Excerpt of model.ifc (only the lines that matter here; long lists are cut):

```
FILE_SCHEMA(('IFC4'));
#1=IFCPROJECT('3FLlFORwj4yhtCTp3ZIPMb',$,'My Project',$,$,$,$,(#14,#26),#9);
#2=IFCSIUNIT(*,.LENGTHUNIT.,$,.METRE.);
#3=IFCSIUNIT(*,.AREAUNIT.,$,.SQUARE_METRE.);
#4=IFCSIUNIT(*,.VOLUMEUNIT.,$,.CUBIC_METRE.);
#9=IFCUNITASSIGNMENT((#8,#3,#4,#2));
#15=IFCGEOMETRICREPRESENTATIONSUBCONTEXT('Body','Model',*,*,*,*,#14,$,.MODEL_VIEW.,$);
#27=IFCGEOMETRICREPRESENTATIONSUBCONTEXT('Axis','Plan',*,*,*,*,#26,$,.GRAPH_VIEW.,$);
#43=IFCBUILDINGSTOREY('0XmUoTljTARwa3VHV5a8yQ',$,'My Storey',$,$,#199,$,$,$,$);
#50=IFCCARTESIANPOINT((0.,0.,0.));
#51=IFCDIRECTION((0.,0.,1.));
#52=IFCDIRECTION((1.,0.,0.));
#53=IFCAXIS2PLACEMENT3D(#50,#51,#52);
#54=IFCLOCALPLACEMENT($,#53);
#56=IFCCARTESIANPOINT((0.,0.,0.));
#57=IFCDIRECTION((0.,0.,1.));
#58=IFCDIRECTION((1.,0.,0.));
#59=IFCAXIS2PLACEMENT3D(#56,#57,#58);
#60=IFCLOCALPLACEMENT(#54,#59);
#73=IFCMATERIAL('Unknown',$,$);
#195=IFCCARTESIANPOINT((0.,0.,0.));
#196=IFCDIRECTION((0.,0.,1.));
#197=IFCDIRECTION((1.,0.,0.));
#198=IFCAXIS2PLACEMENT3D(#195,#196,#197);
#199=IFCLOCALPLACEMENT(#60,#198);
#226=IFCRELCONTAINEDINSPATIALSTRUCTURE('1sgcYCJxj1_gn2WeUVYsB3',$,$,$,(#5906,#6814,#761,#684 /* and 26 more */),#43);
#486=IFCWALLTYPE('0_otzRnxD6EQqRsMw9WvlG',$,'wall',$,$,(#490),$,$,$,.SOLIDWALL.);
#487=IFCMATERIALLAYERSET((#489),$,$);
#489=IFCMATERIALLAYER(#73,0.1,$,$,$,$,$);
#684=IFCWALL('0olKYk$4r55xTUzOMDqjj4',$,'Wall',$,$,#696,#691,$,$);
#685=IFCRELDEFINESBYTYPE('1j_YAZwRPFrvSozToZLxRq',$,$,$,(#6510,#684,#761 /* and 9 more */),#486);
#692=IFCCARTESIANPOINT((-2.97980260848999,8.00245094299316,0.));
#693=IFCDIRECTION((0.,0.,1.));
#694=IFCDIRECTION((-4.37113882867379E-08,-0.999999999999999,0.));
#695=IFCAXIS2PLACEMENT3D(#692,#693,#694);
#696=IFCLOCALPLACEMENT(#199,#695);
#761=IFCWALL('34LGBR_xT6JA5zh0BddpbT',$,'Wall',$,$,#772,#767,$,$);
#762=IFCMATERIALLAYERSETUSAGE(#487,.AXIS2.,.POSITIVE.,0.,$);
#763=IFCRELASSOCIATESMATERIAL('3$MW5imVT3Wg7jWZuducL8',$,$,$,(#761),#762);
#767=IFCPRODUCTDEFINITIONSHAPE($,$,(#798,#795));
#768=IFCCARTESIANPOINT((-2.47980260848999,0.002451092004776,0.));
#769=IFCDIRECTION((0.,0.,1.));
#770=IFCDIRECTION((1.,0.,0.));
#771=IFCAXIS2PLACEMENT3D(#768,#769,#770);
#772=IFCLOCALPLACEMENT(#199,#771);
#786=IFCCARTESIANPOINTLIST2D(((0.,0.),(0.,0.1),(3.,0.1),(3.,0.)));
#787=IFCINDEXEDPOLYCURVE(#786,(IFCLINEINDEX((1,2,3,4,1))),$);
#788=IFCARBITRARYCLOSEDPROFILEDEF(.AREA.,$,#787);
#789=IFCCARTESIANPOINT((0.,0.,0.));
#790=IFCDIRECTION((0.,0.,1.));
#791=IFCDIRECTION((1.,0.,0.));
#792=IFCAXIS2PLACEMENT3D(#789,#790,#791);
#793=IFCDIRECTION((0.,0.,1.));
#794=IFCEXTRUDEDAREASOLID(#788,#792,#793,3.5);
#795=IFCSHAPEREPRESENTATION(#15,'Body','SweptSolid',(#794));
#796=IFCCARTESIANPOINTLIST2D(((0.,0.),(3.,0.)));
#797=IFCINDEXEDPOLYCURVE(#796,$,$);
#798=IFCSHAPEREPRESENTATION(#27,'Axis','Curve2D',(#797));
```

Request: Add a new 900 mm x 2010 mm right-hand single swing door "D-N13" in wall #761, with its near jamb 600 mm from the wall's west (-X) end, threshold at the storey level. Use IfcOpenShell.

```python
import numpy as np
import ifcopenshell
import ifcopenshell.api.feature
import ifcopenshell.api.geometry
import ifcopenshell.api.root
import ifcopenshell.api.spatial
import ifcopenshell.geom
import ifcopenshell.util.element
import ifcopenshell.util.placement
import ifcopenshell.util.representation
import ifcopenshell.util.shape
import ifcopenshell.util.unit

model = ifcopenshell.open("model.ifc")
unit_scale = ifcopenshell.util.unit.calculate_unit_scale(model)
settings = ifcopenshell.geom.settings()


def volume(element):
    """Net volume in cubic metres, openings subtracted."""
    shape = ifcopenshell.geom.create_shape(settings, element)
    return ifcopenshell.util.shape.get_volume(shape.geometry)


wall = model.by_guid("34LGBR_xT6JA5zh0BddpbT")
storey = ifcopenshell.util.element.get_container(wall, ifc_class="IfcBuildingStorey")
context = ifcopenshell.util.representation.get_context(model, "Model", "Body", "MODEL_VIEW")
before = volume(wall)

width, height, from_end, sill = 0.9, 2.01, 0.6, 0.0  # metres

# The wall runs along its own X axis, and the end named is its -X end.
wall_shape = ifcopenshell.geom.create_shape(settings, wall)
x, y, z = ifcopenshell.util.shape.get_vertices(wall_shape.geometry).T
start = x.min() + from_end
face, thickness = float(y.min()), float(y.max() - y.min())
wall_matrix = ifcopenshell.util.placement.get_local_placement(wall.ObjectPlacement)
level = ifcopenshell.util.placement.get_local_placement(storey.ObjectPlacement)[2, 3]


def in_wall(x, y):
    """Placement at x, y metres in the wall's axes, at sill height."""
    matrix = wall_matrix.copy()
    matrix[:, 3] = wall_matrix @ np.array([x / unit_scale, y / unit_scale, 0.0, 1.0])
    matrix[2, 3] = level + sill / unit_scale
    return matrix


# Opening: a box that overshoots both wall faces by 50 mm.
opening = ifcopenshell.api.root.create_entity(model, ifc_class="IfcOpeningElement", predefined_type="OPENING")
box = ifcopenshell.api.geometry.add_wall_representation(
    model, context=context, length=width, height=height, thickness=thickness + 0.1
)
ifcopenshell.api.geometry.assign_representation(model, product=opening, representation=box)
ifcopenshell.api.geometry.edit_object_placement(model, product=opening, matrix=in_wall(start, face - 0.05), is_si=False)
ifcopenshell.api.feature.add_feature(model, feature=opening, element=wall)

door = ifcopenshell.api.root.create_entity(model, ifc_class="IfcDoor", name="D-N13", predefined_type="DOOR")
door.OverallWidth, door.OverallHeight = width / unit_scale, height / unit_scale
door.OperationType = "SINGLE_SWING_RIGHT"
body = ifcopenshell.api.geometry.add_door_representation(
    model,
    context=context,
    overall_width=door.OverallWidth,
    overall_height=door.OverallHeight,
    operation_type="SINGLE_SWING_RIGHT",
    lining_properties={"LiningDepth": thickness / unit_scale, "ThresholdDepth": thickness / unit_scale},
)
ifcopenshell.api.geometry.assign_representation(model, product=door, representation=body)
ifcopenshell.api.spatial.assign_container(model, products=[door], relating_structure=storey)
ifcopenshell.api.feature.add_filling(model, opening=opening, element=door)

# The lining spans the wall, so the door starts at the wall face.
ifcopenshell.api.geometry.edit_object_placement(model, product=door, matrix=in_wall(start, face), is_si=False)

after = volume(wall)

print(f"wall volume {before:.3f} -> {after:.3f} m3")

model.write("model-out.ifc")
```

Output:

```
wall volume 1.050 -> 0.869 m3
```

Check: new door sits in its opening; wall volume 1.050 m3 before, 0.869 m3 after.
